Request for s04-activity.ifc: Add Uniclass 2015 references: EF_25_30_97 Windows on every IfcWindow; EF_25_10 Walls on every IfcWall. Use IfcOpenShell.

First a look at what the model holds.

```python
import ifcopenshell

model = ifcopenshell.open("s04-activity.ifc")
print(model.schema)
print("classifications:", [c.Name for c in model.by_type("IfcClassification")])
for ifc_class in ("IfcDoor", "IfcRoof", "IfcStair", "IfcWall", "IfcWindow"):
    print(ifc_class, len(model.by_type(ifc_class)))
```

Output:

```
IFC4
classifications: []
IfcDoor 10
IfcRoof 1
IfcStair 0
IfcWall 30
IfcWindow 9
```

```python
import ifcopenshell
import ifcopenshell.api.classification

model = ifcopenshell.open("s04-activity.ifc")

system = ifcopenshell.api.classification.add_classification(model, classification="Uniclass 2015")

codes = {
    "IfcWindow": ("EF_25_30_97", "Windows"),
    "IfcWall": ("EF_25_10", "Walls"),
}
for ifc_class, (code, name) in codes.items():
    products = model.by_type(ifc_class)
    ifcopenshell.api.classification.add_reference(
        model, products=products, classification=system, identification=code, name=name
    )
    print(code, len(products))

model.write("s04-activity_v2.ifc")
```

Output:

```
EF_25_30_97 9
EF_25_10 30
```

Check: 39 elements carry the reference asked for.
